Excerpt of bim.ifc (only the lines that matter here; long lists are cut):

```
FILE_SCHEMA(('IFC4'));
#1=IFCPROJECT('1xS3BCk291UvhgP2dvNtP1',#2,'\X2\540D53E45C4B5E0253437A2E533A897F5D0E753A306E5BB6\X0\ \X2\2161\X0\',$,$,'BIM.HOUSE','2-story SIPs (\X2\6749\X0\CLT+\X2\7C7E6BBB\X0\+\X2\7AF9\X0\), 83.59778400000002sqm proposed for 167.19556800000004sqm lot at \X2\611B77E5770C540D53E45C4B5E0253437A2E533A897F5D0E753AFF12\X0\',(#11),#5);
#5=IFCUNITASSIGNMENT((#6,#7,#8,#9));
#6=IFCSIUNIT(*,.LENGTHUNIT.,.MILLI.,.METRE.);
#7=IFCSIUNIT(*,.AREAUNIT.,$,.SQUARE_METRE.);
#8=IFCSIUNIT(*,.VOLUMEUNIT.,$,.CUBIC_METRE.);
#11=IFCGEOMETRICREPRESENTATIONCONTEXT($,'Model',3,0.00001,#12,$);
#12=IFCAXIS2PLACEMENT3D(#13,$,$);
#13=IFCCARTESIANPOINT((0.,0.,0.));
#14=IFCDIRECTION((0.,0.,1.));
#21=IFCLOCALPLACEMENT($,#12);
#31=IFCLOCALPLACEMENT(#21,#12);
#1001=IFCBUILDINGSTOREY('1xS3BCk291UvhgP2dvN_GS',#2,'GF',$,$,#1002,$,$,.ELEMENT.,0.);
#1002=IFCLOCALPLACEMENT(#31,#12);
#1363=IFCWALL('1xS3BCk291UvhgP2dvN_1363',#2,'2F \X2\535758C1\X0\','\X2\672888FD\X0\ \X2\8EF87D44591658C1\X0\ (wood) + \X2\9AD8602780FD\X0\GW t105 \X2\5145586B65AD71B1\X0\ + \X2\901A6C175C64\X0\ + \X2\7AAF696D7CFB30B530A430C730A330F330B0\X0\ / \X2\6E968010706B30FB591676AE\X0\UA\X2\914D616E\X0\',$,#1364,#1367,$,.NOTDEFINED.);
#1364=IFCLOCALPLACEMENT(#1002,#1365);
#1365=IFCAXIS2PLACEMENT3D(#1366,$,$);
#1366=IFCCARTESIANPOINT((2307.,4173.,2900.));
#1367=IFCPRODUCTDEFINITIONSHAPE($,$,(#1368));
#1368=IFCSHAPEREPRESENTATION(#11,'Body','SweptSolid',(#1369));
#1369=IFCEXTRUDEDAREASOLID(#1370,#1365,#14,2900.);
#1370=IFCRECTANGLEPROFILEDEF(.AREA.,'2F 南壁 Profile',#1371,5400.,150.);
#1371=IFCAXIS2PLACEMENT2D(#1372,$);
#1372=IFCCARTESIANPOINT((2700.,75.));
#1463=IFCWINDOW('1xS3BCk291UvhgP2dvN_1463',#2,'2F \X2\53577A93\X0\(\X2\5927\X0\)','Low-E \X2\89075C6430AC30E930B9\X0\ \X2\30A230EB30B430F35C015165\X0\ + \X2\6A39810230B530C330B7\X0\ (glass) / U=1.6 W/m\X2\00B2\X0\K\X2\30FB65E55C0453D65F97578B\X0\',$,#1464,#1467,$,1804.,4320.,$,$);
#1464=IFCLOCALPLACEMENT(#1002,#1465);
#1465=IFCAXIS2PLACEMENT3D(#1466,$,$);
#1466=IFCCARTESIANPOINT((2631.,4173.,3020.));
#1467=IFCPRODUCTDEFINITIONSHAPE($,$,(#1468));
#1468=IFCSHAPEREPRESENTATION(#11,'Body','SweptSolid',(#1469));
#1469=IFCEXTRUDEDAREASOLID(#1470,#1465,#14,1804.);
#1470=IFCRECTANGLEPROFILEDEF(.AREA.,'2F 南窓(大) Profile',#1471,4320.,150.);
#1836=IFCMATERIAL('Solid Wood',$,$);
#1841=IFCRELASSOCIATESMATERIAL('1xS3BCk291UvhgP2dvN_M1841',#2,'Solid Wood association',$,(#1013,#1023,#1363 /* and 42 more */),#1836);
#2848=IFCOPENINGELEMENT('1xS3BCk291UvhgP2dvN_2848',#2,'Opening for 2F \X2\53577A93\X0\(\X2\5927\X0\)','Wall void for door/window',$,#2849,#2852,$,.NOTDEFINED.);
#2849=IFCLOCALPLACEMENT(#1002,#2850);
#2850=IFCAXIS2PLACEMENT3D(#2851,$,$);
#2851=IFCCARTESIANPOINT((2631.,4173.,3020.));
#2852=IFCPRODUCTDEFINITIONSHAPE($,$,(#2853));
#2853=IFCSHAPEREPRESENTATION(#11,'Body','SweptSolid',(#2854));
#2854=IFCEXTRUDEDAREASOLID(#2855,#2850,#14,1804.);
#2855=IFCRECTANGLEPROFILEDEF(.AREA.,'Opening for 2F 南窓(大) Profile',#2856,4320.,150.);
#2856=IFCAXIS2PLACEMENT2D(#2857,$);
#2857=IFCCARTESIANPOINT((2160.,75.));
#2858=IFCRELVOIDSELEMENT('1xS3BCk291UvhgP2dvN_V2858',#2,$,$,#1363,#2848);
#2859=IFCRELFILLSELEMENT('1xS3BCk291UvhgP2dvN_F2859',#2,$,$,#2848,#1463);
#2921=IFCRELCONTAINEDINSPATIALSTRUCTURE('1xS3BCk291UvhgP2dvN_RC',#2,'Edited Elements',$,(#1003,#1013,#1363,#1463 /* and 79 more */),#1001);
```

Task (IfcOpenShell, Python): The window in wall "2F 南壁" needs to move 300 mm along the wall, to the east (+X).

```python
import ifcopenshell
import ifcopenshell.api.geometry
import ifcopenshell.util.placement
import ifcopenshell.util.unit

model = ifcopenshell.open("bim.ifc")
unit_scale = ifcopenshell.util.unit.calculate_unit_scale(model)

window = model.by_guid("1xS3BCk291UvhgP2dvN_1463")
opening = window.FillsVoids[0].RelatingOpeningElement
wall = opening.VoidsElements[0].RelatingBuildingElement

wall_matrix = ifcopenshell.util.placement.get_local_placement(wall.ObjectPlacement)
shift = wall_matrix[:3, 0] * 0.3 / unit_scale
before = ifcopenshell.util.placement.get_local_placement(window.ObjectPlacement)[:3, 3].copy()

# The window is not placed relative to its opening, so move both.
for product in (opening, window):
    matrix = ifcopenshell.util.placement.get_local_placement(product.ObjectPlacement)
    matrix[:3, 3] += shift
    ifcopenshell.api.geometry.edit_object_placement(model, product=product, matrix=matrix, is_si=False)

after = ifcopenshell.util.placement.get_local_placement(window.ObjectPlacement)[:3, 3]
print("window moved by", (after - before).round(3) + 0.0)

model.write("bim_rev.ifc")
```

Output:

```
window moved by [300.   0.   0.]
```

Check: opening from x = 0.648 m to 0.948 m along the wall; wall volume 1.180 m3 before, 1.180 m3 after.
